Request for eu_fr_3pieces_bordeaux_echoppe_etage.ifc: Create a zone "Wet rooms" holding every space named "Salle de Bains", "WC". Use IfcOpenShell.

First a look at what the model holds.

```python
import ifcopenshell

model = ifcopenshell.open("eu_fr_3pieces_bordeaux_echoppe_etage.ifc")
print(model.schema)
seen = {}
for space in model.by_type("IfcSpace"):
    seen[space.LongName] = seen.get(space.LongName, 0) + 1
for name, count in sorted(seen.items(), key=str):
    print(count, "x", name)
print("zones:", [z.Name for z in model.by_type("IfcZone")][:20])
```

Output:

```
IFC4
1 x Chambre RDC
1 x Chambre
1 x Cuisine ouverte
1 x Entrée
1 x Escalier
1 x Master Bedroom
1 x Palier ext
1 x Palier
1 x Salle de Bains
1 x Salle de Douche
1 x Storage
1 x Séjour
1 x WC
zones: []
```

```python
import ifcopenshell
import ifcopenshell.api.group
import ifcopenshell.api.root

model = ifcopenshell.open("eu_fr_3pieces_bordeaux_echoppe_etage.ifc")

names = {"Salle de Bains", "WC"}
spaces = [s for s in model.by_type("IfcSpace") if s.LongName in names]

zone = ifcopenshell.api.root.create_entity(model, ifc_class="IfcZone", name="Wet rooms")
ifcopenshell.api.group.assign_group(model, products=spaces, group=zone)
print(len(spaces), "spaces in", zone.Name)

model.write("eu_fr_3pieces_bordeaux_echoppe_etage_edited.ifc")
```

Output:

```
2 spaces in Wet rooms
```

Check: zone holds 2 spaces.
